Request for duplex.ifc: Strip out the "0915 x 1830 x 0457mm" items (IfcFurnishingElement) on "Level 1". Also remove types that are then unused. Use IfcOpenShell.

First a look at what the model holds.

```python
import ifcopenshell
import ifcopenshell.util.element

model = ifcopenshell.open("duplex.ifc")
print(model.schema)
storey = next(s for s in model.by_type("IfcBuildingStorey") if s.Name == "Level 1")
furniture = [e for e in ifcopenshell.util.element.get_decomposition(storey) if e.is_a("IfcFurnishingElement")]
seen = {}
for e in furniture:
    element_type = ifcopenshell.util.element.get_type(e)
    name = element_type.Name if element_type not in (None, e) else None
    seen[name] = seen.get(name, 0) + 1
for name, count in sorted(seen.items(), key=str):
    print(count, "x", name)
```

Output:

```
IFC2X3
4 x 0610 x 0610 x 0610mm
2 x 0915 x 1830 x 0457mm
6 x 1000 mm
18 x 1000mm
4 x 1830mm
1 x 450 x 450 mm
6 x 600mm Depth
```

```python
import ifcopenshell
import ifcopenshell.api.root
import ifcopenshell.util.element

model = ifcopenshell.open("duplex.ifc")

storey = next(s for s in model.by_type("IfcBuildingStorey") if s.Name == "Level 1")
furniture = [e for e in ifcopenshell.util.element.get_decomposition(storey) if e.is_a("IfcFurnishingElement")]
targets = [e for e in furniture if (t := ifcopenshell.util.element.get_type(e)) not in (None, e) and t.Name == "0915 x 1830 x 0457mm"]
types = {ifcopenshell.util.element.get_type(e) for e in targets} - {None, *targets}

for e in targets:
    ifcopenshell.api.root.remove_product(model, product=e)
print(len(targets), "removed")

unused = [t for t in types if not ifcopenshell.util.element.get_types(t)]
for t in unused:
    ifcopenshell.api.root.remove_product(model, product=t)
print(len(unused), "unused types removed")

model.write("duplex-out.ifc")
```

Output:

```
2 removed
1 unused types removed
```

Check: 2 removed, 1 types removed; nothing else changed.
